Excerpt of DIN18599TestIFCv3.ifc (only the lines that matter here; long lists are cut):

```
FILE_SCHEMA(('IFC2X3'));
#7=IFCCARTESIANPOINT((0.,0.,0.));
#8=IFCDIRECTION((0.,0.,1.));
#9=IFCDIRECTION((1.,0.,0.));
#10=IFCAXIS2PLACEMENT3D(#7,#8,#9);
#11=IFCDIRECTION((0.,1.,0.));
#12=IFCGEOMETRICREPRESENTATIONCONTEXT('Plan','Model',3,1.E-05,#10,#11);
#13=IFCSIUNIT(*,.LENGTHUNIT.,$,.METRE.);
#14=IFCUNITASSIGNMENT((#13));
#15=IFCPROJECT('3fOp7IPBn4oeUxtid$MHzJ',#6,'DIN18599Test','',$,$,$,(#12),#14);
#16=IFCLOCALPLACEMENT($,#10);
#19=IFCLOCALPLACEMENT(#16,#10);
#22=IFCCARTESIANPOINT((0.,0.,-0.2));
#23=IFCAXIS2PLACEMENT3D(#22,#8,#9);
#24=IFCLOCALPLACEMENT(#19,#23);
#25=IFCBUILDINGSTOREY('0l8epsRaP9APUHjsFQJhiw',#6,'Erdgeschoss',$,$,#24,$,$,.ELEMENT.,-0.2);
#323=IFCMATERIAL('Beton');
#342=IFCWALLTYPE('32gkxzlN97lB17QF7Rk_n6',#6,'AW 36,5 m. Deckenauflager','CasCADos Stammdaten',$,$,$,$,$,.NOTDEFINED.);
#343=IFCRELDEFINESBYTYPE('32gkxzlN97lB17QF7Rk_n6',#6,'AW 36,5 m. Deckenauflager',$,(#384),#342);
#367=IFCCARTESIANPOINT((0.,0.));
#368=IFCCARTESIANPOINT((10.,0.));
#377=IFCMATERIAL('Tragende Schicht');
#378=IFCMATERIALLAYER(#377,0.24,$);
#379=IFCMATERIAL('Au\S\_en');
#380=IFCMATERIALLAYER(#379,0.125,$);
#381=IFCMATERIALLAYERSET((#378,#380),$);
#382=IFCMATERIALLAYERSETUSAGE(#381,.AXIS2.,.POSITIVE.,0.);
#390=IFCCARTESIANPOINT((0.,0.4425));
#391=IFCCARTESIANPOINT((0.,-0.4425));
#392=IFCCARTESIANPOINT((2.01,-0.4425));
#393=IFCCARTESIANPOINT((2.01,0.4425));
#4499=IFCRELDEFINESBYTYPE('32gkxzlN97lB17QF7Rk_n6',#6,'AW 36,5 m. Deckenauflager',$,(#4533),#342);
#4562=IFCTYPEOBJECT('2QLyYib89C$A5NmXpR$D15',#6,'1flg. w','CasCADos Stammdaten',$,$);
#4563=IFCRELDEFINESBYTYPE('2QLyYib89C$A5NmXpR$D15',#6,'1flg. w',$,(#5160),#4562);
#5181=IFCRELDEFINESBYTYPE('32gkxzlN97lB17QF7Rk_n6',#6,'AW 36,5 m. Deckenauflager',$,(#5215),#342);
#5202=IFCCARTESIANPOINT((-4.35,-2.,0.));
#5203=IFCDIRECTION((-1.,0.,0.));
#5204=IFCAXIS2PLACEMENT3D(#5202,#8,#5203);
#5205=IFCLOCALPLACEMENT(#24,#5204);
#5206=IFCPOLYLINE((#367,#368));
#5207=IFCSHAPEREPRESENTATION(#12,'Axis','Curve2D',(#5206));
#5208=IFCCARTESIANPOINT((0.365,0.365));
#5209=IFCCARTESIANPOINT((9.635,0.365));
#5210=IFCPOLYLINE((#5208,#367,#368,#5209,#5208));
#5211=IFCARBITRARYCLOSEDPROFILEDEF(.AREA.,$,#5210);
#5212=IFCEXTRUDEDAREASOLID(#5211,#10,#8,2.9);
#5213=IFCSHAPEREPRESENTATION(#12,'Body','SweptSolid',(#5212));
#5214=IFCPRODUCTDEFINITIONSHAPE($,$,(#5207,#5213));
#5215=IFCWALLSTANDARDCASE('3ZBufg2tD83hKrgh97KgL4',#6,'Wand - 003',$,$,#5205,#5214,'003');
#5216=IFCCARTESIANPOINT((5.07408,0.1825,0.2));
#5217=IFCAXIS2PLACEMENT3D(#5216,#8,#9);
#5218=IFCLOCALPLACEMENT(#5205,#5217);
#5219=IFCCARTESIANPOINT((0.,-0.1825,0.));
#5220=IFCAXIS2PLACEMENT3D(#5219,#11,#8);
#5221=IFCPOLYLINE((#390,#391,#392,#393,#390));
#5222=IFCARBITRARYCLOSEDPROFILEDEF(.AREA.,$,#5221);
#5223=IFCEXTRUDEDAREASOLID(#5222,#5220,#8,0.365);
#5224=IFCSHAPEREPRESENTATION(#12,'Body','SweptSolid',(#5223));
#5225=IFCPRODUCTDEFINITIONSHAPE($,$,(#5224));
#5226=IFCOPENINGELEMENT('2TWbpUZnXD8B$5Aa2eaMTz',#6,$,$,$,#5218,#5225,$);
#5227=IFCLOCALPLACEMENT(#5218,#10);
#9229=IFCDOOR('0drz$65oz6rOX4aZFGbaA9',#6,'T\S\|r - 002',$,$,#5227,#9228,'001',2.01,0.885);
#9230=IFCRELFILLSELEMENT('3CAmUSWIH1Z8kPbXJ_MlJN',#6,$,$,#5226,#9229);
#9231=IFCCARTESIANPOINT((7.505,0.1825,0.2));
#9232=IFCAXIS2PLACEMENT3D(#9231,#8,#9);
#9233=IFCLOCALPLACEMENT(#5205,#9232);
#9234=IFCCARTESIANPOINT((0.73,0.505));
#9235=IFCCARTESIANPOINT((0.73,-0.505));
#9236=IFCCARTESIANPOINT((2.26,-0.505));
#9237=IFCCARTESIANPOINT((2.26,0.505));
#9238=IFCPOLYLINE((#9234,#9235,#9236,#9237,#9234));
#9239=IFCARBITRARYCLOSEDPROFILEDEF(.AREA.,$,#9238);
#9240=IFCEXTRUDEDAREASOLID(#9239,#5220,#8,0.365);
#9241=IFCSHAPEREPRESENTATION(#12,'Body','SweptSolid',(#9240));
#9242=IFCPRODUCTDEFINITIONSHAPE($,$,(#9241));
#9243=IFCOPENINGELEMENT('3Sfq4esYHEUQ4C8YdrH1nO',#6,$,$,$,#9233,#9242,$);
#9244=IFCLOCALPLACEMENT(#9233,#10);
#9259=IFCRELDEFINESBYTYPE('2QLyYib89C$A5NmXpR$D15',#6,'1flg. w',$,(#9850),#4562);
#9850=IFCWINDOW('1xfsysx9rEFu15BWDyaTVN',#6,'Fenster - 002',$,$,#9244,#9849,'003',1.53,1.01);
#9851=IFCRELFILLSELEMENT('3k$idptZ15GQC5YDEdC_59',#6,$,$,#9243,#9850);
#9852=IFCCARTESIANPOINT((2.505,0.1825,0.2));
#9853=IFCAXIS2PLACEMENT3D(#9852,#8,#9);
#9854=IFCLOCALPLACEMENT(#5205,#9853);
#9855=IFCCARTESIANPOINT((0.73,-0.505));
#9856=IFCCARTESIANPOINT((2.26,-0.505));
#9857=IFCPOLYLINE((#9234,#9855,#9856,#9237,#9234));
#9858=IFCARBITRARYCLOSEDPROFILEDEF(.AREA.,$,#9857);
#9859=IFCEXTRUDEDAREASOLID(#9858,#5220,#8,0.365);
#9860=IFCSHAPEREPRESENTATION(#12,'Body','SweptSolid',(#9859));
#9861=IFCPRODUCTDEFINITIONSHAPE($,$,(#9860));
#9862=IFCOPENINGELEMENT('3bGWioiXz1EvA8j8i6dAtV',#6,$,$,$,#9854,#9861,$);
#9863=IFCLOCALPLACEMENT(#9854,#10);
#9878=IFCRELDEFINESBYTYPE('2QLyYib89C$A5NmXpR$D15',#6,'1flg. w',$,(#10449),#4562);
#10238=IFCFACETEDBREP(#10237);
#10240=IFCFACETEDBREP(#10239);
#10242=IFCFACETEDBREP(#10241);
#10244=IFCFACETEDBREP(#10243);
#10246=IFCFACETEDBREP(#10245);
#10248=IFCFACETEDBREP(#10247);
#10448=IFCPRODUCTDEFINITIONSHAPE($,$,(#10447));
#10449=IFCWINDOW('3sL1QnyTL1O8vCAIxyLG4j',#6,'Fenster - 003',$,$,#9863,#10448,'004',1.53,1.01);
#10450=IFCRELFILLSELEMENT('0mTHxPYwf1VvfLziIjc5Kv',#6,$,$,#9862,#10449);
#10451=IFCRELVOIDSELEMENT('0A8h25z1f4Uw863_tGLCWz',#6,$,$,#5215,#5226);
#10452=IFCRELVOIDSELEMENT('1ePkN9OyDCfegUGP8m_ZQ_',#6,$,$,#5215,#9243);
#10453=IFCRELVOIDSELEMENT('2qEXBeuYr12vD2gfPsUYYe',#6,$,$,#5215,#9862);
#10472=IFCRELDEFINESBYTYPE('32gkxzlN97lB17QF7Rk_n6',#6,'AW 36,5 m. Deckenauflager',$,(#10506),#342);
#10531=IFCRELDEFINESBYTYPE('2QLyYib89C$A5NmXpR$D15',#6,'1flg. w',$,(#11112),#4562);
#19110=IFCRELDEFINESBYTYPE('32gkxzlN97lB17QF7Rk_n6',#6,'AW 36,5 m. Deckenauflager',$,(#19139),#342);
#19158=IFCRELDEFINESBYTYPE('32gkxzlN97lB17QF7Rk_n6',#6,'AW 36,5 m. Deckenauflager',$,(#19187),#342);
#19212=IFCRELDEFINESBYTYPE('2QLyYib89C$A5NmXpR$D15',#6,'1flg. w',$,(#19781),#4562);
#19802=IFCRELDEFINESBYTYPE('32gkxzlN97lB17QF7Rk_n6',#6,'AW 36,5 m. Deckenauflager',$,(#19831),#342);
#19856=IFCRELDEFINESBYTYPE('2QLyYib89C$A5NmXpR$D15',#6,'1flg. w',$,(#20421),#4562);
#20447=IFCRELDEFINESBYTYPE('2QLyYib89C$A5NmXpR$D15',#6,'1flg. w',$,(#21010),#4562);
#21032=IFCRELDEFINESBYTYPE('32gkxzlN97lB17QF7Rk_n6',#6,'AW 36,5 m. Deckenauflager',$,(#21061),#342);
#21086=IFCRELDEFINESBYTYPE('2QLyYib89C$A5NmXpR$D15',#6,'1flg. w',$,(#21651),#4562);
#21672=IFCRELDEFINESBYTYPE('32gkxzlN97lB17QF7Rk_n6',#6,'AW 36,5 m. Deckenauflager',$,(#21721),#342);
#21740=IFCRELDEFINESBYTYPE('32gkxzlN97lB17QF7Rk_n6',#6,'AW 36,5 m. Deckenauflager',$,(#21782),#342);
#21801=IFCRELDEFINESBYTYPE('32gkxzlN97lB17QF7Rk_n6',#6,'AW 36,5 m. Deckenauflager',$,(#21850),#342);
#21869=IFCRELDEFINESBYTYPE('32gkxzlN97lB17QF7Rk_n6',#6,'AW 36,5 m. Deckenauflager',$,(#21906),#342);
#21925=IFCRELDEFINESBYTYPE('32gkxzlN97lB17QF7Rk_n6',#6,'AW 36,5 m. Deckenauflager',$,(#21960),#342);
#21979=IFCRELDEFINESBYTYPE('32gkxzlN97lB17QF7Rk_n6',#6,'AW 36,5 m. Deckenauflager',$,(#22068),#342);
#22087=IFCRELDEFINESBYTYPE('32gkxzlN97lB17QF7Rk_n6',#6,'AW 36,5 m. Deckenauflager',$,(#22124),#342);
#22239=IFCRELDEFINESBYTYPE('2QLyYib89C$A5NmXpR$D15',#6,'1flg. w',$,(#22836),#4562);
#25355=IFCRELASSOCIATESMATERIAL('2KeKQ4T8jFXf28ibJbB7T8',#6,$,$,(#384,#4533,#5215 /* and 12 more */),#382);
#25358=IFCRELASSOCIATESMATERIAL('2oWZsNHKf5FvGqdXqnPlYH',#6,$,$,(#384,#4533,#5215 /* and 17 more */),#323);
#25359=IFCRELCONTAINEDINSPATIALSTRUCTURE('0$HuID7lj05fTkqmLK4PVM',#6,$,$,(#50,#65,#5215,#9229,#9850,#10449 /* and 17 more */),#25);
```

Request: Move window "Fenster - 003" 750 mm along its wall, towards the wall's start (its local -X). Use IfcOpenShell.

```python
import ifcopenshell
import ifcopenshell.api.geometry
import ifcopenshell.util.placement

model = ifcopenshell.open("DIN18599TestIFCv3.ifc")

window = model.by_id(10449)
opening = window.FillsVoids[0].RelatingOpeningElement
wall = opening.VoidsElements[0].RelatingBuildingElement

wall_matrix = ifcopenshell.util.placement.get_local_placement(wall.ObjectPlacement)
shift = wall_matrix[:3, 0] * -0.75
before = ifcopenshell.util.placement.get_local_placement(window.ObjectPlacement)[:3, 3].copy()

# The window is placed relative to its opening, so it follows when the opening moves.
matrix = ifcopenshell.util.placement.get_local_placement(opening.ObjectPlacement)
matrix[:3, 3] += shift
ifcopenshell.api.geometry.edit_object_placement(
    model, product=opening, matrix=matrix, is_si=False, should_transform_children=True
)

after = ifcopenshell.util.placement.get_local_placement(window.ObjectPlacement)[:3, 3]
print("window moved by", (after - before).round(3) + 0.0)

model.write("DIN18599TestIFCv3_updated.ifc")
```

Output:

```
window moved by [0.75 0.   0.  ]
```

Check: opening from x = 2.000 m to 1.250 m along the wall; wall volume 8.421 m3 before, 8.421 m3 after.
